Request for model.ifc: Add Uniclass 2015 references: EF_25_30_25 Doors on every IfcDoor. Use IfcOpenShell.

First a look at what the model holds.

```python
import ifcopenshell

model = ifcopenshell.open("model.ifc")
print(model.schema)
print("classifications:", [c.Name for c in model.by_type("IfcClassification")])
for ifc_class in ("IfcDoor", "IfcRoof", "IfcStair", "IfcWall", "IfcWindow"):
    print(ifc_class, len(model.by_type(ifc_class)))
```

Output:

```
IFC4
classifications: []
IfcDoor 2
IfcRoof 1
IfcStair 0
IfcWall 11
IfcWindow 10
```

```python
import ifcopenshell
import ifcopenshell.api.classification

model = ifcopenshell.open("model.ifc")

system = ifcopenshell.api.classification.add_classification(model, classification="Uniclass 2015")

codes = {
    "IfcDoor": ("EF_25_30_25", "Doors"),
}
for ifc_class, (code, name) in codes.items():
    products = model.by_type(ifc_class)
    ifcopenshell.api.classification.add_reference(
        model, products=products, classification=system, identification=code, name=name
    )
    print(code, len(products))

model.write("model_rev.ifc")
```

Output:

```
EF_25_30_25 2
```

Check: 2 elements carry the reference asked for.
